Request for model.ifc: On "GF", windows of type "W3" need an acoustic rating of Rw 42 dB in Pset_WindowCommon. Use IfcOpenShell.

First a look at what the model holds.

```python
import ifcopenshell
import ifcopenshell.util.element

model = ifcopenshell.open("model.ifc")
print(model.schema)
storey = next(s for s in model.by_type("IfcBuildingStorey") if s.Name == "GF")
windows = [e for e in ifcopenshell.util.element.get_decomposition(storey) if e.is_a("IfcWindow")]
seen = {}
for e in windows:
    element_type = ifcopenshell.util.element.get_type(e)
    key = (element_type.Name if element_type != e and element_type else None, ifcopenshell.util.element.get_pset(e, "Pset_WindowCommon", "AcousticRating"))
    seen[key] = seen.get(key, 0) + 1
for (name, value), count in sorted(seen.items(), key=str):
    print(count, "x", name, "|", value)
```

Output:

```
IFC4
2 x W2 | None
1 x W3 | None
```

```python
import ifcopenshell
import ifcopenshell.api.pset
import ifcopenshell.util.element

model = ifcopenshell.open("model.ifc")

storey = next(s for s in model.by_type("IfcBuildingStorey") if s.Name == "GF")
windows = [e for e in ifcopenshell.util.element.get_decomposition(storey) if e.is_a("IfcWindow")]

count = 0
for e in windows:
    element_type = ifcopenshell.util.element.get_type(e)
    if element_type in (None, e) or element_type.Name != "W3":
        continue
    # add_pset returns the element's existing set when there is one.
    pset = ifcopenshell.api.pset.add_pset(model, product=e, name="Pset_WindowCommon")
    ifcopenshell.api.pset.edit_pset(model, pset=pset, properties={"AcousticRating": "Rw 42 dB"})
    count += 1

print(count, "windows updated")

model.write("model-out.ifc")
```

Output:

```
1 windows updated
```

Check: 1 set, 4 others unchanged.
